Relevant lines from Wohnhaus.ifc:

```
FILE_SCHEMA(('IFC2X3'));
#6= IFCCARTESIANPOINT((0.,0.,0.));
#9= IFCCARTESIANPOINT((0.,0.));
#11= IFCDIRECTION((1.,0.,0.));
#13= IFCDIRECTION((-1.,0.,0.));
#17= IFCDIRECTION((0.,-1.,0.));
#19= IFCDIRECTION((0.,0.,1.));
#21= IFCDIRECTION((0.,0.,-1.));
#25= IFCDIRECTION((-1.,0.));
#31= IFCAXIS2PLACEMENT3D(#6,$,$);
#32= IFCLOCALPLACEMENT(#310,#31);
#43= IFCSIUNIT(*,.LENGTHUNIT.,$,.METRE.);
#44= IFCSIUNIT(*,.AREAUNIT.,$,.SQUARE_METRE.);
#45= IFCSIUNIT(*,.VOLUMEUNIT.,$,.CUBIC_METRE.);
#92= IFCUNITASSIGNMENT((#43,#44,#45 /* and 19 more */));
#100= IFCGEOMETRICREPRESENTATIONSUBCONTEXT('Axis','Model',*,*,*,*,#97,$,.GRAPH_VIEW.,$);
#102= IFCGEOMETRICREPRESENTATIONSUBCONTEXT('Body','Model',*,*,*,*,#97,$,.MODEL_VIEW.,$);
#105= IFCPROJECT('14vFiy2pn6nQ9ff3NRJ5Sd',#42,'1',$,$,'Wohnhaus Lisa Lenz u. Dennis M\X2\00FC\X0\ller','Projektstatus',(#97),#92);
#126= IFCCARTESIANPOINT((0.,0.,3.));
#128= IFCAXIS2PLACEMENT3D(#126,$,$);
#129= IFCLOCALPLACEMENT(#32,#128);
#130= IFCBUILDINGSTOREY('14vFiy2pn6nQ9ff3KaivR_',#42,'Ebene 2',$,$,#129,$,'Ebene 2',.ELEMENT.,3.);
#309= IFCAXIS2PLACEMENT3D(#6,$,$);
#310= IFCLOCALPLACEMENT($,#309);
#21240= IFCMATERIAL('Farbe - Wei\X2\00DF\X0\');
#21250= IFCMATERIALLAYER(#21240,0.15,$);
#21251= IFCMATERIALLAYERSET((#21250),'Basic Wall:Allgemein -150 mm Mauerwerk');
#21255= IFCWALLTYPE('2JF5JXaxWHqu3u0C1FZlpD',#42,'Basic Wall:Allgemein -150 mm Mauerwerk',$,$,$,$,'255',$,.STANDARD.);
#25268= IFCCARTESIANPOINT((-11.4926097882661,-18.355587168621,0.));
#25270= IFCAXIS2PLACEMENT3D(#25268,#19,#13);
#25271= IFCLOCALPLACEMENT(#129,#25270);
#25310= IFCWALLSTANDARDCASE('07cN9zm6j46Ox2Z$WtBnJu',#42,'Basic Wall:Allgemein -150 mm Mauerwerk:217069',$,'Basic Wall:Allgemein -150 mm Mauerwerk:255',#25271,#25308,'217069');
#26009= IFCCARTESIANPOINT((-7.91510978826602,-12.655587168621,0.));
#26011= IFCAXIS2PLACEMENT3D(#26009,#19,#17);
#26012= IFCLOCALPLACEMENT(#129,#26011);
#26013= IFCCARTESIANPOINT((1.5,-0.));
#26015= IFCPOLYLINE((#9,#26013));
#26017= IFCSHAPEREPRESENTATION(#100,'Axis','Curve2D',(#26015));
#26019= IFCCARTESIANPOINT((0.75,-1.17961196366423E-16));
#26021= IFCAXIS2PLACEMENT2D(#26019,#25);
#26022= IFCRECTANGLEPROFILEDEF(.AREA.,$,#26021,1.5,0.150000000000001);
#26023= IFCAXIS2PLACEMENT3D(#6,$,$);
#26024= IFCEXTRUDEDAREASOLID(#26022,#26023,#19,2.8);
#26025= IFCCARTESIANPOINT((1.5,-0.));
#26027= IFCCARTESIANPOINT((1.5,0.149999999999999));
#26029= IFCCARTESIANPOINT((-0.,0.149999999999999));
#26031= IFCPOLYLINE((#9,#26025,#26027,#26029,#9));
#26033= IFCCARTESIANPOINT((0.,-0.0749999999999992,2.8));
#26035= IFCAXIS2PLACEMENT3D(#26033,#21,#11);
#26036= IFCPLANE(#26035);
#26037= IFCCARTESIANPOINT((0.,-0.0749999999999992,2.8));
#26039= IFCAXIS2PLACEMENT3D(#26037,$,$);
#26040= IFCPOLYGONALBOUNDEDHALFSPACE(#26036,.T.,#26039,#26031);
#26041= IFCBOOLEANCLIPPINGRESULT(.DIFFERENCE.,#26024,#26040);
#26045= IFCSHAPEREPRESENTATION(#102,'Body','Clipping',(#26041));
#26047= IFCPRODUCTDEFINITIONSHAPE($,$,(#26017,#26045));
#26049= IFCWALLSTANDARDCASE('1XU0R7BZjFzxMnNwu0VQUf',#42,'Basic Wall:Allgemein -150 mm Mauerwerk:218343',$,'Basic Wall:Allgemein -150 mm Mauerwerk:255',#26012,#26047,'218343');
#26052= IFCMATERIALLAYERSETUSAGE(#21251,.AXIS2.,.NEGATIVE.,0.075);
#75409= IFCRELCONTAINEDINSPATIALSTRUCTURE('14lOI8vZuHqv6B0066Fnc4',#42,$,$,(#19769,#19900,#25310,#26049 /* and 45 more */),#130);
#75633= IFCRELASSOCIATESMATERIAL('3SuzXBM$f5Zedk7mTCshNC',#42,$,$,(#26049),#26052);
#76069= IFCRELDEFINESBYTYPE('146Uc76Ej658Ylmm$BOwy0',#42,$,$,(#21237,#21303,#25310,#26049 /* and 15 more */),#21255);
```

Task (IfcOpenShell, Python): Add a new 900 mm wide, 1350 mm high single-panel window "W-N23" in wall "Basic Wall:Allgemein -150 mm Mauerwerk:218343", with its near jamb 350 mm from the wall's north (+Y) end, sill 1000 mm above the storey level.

```python
import numpy as np
import ifcopenshell
import ifcopenshell.api.feature
import ifcopenshell.api.geometry
import ifcopenshell.api.root
import ifcopenshell.api.spatial
import ifcopenshell.api.type
import ifcopenshell.geom
import ifcopenshell.util.element
import ifcopenshell.util.placement
import ifcopenshell.util.representation
import ifcopenshell.util.shape
import ifcopenshell.util.unit

model = ifcopenshell.open("Wohnhaus.ifc")
unit_scale = ifcopenshell.util.unit.calculate_unit_scale(model)
settings = ifcopenshell.geom.settings()


def volume(element):
    """Net volume in cubic metres, openings subtracted."""
    shape = ifcopenshell.geom.create_shape(settings, element)
    return ifcopenshell.util.shape.get_volume(shape.geometry)


wall = model.by_id(26049)
storey = ifcopenshell.util.element.get_container(wall, ifc_class="IfcBuildingStorey")
context = ifcopenshell.util.representation.get_context(model, "Model", "Body", "MODEL_VIEW")
before = volume(wall)

width, height, from_end, sill = 0.9, 1.35, 0.35, 1  # metres

# The wall runs along its own X axis, and the end named is its -X end.
wall_shape = ifcopenshell.geom.create_shape(settings, wall)
x, y, z = ifcopenshell.util.shape.get_vertices(wall_shape.geometry).T
start = x.min() + from_end
face, thickness = float(y.min()), float(y.max() - y.min())
wall_matrix = ifcopenshell.util.placement.get_local_placement(wall.ObjectPlacement)
level = ifcopenshell.util.placement.get_local_placement(storey.ObjectPlacement)[2, 3]


def in_wall(x, y):
    """Placement at x, y metres in the wall's axes, at sill height."""
    matrix = wall_matrix.copy()
    matrix[:, 3] = wall_matrix @ np.array([x / unit_scale, y / unit_scale, 0.0, 1.0])
    matrix[2, 3] = level + sill / unit_scale
    return matrix


# Opening: a box that overshoots both wall faces by 50 mm.
opening = ifcopenshell.api.root.create_entity(model, ifc_class="IfcOpeningElement")
box = ifcopenshell.api.geometry.add_wall_representation(
    model, context=context, length=width, height=height, thickness=thickness + 0.1
)
ifcopenshell.api.geometry.assign_representation(model, product=opening, representation=box)
ifcopenshell.api.geometry.edit_object_placement(model, product=opening, matrix=in_wall(start, face - 0.05), is_si=False)
ifcopenshell.api.feature.add_feature(model, feature=opening, element=wall)

window = ifcopenshell.api.root.create_entity(model, ifc_class="IfcWindow", name="W-N23")
window.OverallWidth, window.OverallHeight = width / unit_scale, height / unit_scale
body = ifcopenshell.api.geometry.add_window_representation(
    model,
    context=context,
    overall_width=window.OverallWidth,
    overall_height=window.OverallHeight,
    partition_type="SINGLE_PANEL",
)
ifcopenshell.api.geometry.assign_representation(model, product=window, representation=body)
ifcopenshell.api.spatial.assign_container(model, products=[window], relating_structure=storey)
fills = ifcopenshell.api.feature.add_filling(model, opening=opening, element=window)
fills.OwnerHistory = window.OwnerHistory  # required in IFC2X3

# IFC2X3 keeps the operation on the window style.
style = ifcopenshell.api.root.create_entity(model, ifc_class="IfcWindowStyle", name="W-N23")
style.OperationType, style.ConstructionType = "SINGLE_PANEL", "NOTDEFINED"
style.ParameterTakesPrecedence = style.Sizeable = False
ifcopenshell.api.type.assign_type(model, related_objects=[window], relating_type=style)

# Centre the window in the wall's thickness.
ifcopenshell.api.geometry.edit_object_placement(model, product=window, matrix=in_wall(start, face), is_si=False)
window_shape = ifcopenshell.geom.create_shape(settings, window)
depth = ifcopenshell.util.shape.get_vertices(window_shape.geometry)[:, 1]
offset = face + thickness / 2 - (depth.min() + depth.max()) / 2
ifcopenshell.api.geometry.edit_object_placement(model, product=window, matrix=in_wall(start, offset), is_si=False)

after = volume(wall)

print(f"wall volume {before:.3f} -> {after:.3f} m3")

model.write("Wohnhaus_edited.ifc")
```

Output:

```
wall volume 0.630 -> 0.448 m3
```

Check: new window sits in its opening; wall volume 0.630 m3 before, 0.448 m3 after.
